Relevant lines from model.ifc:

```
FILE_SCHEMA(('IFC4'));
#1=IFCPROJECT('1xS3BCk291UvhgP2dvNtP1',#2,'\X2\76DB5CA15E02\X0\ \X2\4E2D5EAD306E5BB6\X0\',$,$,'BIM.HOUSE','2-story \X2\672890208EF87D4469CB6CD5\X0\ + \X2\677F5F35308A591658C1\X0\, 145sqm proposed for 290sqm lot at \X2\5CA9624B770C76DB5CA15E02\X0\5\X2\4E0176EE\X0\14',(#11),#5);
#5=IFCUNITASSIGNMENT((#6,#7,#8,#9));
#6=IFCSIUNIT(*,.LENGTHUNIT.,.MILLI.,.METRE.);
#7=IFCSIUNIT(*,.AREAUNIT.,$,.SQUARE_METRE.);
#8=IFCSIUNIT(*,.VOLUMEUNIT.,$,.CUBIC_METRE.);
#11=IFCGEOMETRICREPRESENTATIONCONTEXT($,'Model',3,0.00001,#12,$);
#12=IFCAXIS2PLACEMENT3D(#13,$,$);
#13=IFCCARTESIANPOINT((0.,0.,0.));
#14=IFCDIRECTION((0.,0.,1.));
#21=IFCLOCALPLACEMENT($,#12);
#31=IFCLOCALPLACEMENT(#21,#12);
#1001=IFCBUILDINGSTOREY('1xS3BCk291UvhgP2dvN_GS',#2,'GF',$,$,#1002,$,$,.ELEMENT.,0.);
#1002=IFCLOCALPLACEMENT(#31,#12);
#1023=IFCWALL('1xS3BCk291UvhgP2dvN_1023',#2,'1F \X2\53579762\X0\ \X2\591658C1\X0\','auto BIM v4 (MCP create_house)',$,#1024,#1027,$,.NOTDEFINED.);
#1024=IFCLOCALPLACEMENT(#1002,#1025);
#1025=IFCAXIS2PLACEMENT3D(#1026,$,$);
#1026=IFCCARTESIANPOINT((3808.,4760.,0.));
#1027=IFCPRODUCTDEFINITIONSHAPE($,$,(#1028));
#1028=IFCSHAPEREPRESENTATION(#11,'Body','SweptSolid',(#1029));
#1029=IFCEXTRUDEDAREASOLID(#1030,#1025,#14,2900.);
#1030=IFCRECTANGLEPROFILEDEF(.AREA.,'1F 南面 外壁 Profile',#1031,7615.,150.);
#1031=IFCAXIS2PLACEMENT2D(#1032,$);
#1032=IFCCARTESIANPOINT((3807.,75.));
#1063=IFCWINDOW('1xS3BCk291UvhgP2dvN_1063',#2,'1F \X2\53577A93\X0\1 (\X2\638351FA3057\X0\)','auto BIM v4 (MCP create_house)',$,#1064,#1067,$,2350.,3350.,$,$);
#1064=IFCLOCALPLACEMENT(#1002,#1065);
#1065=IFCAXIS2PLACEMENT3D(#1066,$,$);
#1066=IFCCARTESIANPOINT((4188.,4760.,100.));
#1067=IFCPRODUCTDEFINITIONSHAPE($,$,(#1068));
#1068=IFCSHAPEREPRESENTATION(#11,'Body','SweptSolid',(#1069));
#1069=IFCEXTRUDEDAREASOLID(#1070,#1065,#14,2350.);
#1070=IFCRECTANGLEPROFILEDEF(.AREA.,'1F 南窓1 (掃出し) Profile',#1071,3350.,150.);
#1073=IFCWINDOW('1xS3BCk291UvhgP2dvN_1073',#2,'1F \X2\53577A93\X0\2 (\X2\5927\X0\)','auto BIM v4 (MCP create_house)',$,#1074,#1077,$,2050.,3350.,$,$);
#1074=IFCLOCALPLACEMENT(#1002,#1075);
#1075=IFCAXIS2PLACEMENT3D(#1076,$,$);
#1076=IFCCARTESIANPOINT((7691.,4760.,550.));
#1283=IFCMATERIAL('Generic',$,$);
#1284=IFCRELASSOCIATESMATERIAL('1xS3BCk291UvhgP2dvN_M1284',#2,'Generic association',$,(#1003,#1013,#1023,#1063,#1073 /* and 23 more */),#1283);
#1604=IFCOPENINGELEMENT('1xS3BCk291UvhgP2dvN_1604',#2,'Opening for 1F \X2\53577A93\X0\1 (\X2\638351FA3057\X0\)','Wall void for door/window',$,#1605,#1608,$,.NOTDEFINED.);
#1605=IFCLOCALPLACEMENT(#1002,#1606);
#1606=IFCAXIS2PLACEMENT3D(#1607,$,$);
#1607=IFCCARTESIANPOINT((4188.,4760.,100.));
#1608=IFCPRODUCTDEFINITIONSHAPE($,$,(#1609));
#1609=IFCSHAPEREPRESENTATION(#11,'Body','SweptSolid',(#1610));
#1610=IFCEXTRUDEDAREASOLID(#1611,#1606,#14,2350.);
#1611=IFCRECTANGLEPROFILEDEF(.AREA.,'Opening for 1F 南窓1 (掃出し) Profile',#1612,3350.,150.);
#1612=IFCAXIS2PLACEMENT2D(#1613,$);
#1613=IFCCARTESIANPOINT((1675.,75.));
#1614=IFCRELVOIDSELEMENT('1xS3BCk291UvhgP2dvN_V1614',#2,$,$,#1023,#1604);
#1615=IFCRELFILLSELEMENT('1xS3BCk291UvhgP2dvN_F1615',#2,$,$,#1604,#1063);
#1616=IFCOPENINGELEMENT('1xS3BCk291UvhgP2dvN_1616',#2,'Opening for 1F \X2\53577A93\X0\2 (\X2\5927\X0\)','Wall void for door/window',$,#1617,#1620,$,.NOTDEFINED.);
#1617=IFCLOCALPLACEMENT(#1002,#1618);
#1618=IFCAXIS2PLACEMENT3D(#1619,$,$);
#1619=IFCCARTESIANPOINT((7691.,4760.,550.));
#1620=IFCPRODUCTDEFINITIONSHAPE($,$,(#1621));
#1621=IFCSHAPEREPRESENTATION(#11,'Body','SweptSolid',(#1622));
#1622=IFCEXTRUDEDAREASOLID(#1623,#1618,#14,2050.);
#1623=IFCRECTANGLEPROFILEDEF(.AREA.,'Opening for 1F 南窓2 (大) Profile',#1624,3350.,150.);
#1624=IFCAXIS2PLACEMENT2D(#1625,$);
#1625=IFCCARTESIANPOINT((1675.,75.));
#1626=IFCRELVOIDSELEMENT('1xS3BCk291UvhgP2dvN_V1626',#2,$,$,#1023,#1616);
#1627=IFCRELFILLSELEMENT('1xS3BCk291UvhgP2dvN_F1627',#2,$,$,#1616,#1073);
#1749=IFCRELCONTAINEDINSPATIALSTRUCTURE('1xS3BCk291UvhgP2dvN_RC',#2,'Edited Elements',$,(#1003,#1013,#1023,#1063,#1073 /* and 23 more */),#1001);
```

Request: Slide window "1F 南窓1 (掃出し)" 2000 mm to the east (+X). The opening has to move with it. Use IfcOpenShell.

```python
import ifcopenshell
import ifcopenshell.api.geometry
import ifcopenshell.util.placement

model = ifcopenshell.open("model.ifc")

window = model.by_guid("1xS3BCk291UvhgP2dvN_1063")
opening = window.FillsVoids[0].RelatingOpeningElement
wall = opening.VoidsElements[0].RelatingBuildingElement

wall_matrix = ifcopenshell.util.placement.get_local_placement(wall.ObjectPlacement)
shift = wall_matrix[:3, 0] * 2000.0
before = ifcopenshell.util.placement.get_local_placement(window.ObjectPlacement)[:3, 3].copy()

# The window is not placed relative to its opening, so move both.
for product in (opening, window):
    matrix = ifcopenshell.util.placement.get_local_placement(product.ObjectPlacement)
    matrix[:3, 3] += shift
    ifcopenshell.api.geometry.edit_object_placement(model, product=product, matrix=matrix, is_si=False)

after = ifcopenshell.util.placement.get_local_placement(window.ObjectPlacement)[:3, 3]
print("window moved by", (after - before).round(3) + 0.0)

model.write("model_v2.ifc")
```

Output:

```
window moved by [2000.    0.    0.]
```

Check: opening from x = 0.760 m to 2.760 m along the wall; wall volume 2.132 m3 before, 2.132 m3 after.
